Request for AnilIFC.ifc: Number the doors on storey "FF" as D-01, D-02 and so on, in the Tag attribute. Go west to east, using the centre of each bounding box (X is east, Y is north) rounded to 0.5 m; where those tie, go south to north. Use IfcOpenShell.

First a look at what the model holds.

```python
import ifcopenshell
import ifcopenshell.util.element
import ifcopenshell.util.placement

model = ifcopenshell.open("AnilIFC.ifc")
print(model.schema)
storey = next(s for s in model.by_type("IfcBuildingStorey") if s.Name == "FF")
doors = [e for e in ifcopenshell.util.element.get_decomposition(storey) if e.is_a("IfcDoor")]
for e in sorted(doors, key=lambda e: e.id()):
    origin = ifcopenshell.util.placement.get_local_placement(e.ObjectPlacement)[:3, 3]
    print(e.id(), e.Tag, e.Name, origin.round(2) + 0.0, sep=" | ")
```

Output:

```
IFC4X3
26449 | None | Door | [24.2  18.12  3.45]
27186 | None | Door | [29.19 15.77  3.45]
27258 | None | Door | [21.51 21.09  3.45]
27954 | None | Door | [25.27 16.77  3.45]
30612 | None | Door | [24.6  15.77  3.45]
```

```python
import ifcopenshell
import ifcopenshell.geom
import ifcopenshell.util.element
import ifcopenshell.util.shape

model = ifcopenshell.open("AnilIFC.ifc")
settings = ifcopenshell.geom.settings()
settings.set("use-world-coords", True)


def centre(element):
    shape = ifcopenshell.geom.create_shape(settings, element)
    return ifcopenshell.util.shape.get_bbox_centroid(shape.geometry)


storey = next(s for s in model.by_type("IfcBuildingStorey") if s.Name == "FF")
doors = [e for e in ifcopenshell.util.element.get_decomposition(storey) if e.is_a("IfcDoor")]

# Insertion points can sit at a corner or the storey origin, so sort by the geometry (in metres).
centres = {e: centre(e) for e in doors}
doors.sort(key=lambda e: (round(centres[e][0] / 0.5), centres[e][1]))

for i, e in enumerate(doors, start=1):
    number = f"D-{i:02d}"
    e.Tag = number
    print(e.id(), number)

model.write("AnilIFC_rev.ifc")
```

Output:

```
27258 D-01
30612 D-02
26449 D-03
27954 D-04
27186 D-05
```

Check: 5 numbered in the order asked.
